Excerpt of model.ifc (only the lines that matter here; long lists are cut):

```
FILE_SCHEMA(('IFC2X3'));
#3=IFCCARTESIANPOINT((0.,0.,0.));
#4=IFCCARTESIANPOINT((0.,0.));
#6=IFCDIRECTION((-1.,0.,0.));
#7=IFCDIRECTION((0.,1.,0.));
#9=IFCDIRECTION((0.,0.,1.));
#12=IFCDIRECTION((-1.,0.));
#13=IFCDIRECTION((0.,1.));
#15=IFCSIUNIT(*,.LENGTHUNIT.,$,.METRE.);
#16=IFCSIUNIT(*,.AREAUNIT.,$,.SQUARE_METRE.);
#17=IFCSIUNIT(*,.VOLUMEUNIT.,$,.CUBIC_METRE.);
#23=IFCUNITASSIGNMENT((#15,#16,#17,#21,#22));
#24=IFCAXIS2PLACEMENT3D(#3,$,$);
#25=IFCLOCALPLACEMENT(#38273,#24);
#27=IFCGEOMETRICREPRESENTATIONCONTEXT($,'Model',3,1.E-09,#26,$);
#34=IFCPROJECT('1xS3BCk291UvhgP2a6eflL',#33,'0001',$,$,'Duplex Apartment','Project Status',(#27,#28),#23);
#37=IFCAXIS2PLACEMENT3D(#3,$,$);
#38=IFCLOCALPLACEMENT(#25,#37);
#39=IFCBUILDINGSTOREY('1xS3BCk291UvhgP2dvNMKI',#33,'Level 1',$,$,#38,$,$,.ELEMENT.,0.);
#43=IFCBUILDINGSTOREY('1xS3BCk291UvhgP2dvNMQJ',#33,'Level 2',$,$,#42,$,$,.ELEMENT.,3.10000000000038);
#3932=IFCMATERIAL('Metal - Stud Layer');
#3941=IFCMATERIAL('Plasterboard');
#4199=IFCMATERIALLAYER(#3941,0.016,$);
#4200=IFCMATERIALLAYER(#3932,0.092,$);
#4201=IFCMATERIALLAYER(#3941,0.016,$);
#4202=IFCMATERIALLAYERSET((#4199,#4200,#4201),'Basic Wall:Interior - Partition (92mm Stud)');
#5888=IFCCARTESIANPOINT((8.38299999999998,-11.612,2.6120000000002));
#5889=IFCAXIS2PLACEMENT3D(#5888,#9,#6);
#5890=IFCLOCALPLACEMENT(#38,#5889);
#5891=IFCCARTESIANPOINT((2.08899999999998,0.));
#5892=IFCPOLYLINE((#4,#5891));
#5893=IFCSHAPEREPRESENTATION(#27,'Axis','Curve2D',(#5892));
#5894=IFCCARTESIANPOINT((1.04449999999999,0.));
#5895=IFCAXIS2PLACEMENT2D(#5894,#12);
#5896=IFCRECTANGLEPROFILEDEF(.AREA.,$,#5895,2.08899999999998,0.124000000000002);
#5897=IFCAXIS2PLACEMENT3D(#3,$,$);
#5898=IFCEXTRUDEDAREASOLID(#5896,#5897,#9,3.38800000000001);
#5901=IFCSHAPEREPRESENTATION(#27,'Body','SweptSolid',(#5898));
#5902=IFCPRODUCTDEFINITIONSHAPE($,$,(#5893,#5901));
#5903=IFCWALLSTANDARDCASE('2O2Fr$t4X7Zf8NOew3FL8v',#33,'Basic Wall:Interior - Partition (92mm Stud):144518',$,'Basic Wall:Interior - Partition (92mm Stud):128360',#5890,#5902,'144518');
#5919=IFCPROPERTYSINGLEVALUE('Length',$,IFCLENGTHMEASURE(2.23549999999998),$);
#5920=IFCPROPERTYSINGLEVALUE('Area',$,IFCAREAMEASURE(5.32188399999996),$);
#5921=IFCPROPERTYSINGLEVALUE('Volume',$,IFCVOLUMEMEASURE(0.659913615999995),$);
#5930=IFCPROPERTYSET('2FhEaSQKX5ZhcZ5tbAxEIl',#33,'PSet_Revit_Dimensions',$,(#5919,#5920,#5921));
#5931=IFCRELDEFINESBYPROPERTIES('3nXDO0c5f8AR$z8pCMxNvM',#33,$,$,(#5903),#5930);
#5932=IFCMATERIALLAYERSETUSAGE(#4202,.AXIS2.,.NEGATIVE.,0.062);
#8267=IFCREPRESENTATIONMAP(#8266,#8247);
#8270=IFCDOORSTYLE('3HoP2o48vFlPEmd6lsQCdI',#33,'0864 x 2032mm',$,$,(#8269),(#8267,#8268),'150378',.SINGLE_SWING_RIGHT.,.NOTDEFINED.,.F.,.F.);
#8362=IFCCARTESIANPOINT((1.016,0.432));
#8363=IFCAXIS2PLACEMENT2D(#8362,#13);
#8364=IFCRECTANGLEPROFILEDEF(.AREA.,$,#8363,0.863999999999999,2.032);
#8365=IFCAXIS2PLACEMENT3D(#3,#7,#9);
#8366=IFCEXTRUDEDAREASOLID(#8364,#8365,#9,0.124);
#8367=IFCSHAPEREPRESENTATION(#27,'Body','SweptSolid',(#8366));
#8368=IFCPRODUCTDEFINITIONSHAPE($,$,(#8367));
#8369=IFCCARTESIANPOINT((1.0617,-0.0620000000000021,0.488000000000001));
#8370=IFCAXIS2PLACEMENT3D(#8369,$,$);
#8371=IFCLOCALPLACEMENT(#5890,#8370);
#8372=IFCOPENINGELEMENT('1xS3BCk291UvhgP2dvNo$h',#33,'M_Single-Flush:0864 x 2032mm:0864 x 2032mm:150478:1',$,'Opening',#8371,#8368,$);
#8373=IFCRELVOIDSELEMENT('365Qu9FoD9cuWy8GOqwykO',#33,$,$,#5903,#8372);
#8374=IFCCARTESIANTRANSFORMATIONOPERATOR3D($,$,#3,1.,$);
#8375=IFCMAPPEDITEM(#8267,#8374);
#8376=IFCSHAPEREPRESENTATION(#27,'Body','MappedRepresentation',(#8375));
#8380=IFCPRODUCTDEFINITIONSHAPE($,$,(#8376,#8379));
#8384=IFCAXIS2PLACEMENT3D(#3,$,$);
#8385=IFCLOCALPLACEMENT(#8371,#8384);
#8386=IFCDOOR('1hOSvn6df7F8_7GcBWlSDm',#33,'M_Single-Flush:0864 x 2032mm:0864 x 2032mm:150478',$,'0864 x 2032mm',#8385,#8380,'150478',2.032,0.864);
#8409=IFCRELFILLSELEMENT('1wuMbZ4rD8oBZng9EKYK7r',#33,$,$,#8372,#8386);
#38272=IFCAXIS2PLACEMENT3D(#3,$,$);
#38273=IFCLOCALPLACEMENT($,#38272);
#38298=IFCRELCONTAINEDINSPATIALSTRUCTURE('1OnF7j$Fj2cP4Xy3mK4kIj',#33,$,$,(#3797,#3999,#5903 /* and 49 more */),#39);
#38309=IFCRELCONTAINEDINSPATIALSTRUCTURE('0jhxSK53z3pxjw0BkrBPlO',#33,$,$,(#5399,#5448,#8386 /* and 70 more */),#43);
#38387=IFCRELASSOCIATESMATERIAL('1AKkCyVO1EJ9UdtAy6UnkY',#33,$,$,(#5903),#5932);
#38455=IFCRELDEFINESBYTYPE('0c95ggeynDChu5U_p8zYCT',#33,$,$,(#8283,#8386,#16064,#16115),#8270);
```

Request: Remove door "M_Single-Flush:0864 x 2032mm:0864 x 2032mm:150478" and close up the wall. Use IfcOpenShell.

```python
import ifcopenshell
import ifcopenshell.api.feature
import ifcopenshell.api.pset
import ifcopenshell.api.root
import ifcopenshell.geom
import ifcopenshell.util.element
import ifcopenshell.util.shape
import ifcopenshell.util.unit

model = ifcopenshell.open("model.ifc")
area_scale = ifcopenshell.util.unit.calculate_unit_scale(model, "AREAUNIT")
volume_scale = ifcopenshell.util.unit.calculate_unit_scale(model, "VOLUMEUNIT")
settings = ifcopenshell.geom.settings()


def volume(element):
    """Net volume in cubic metres, openings subtracted."""
    shape = ifcopenshell.geom.create_shape(settings, element)
    return ifcopenshell.util.shape.get_volume(shape.geometry)


door = model.by_guid("1hOSvn6df7F8_7GcBWlSDm")
opening = door.FillsVoids[0].RelatingOpeningElement
wall = opening.VoidsElements[0].RelatingBuildingElement
before = volume(wall)

ifcopenshell.api.root.remove_product(model, product=door)
ifcopenshell.api.feature.remove_feature(model, feature=opening)

after = volume(wall)
thickness = 0.124  # wall thickness in metres

# Update the wall's stored quantities.
pset = model.by_id(ifcopenshell.util.element.get_pset(wall, "PSet_Revit_Dimensions", should_inherit=False)["id"])
ifcopenshell.api.pset.edit_pset(model, pset=pset, properties={
    "Area": model.create_entity("IfcAreaMeasure", after / thickness / area_scale),
    "Volume": model.create_entity("IfcVolumeMeasure", after / volume_scale),
})

print(f"wall volume {before:.3f} -> {after:.3f} m3")

model.write("model_v2.ifc")
```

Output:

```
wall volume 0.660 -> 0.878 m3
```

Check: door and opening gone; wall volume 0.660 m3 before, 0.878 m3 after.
